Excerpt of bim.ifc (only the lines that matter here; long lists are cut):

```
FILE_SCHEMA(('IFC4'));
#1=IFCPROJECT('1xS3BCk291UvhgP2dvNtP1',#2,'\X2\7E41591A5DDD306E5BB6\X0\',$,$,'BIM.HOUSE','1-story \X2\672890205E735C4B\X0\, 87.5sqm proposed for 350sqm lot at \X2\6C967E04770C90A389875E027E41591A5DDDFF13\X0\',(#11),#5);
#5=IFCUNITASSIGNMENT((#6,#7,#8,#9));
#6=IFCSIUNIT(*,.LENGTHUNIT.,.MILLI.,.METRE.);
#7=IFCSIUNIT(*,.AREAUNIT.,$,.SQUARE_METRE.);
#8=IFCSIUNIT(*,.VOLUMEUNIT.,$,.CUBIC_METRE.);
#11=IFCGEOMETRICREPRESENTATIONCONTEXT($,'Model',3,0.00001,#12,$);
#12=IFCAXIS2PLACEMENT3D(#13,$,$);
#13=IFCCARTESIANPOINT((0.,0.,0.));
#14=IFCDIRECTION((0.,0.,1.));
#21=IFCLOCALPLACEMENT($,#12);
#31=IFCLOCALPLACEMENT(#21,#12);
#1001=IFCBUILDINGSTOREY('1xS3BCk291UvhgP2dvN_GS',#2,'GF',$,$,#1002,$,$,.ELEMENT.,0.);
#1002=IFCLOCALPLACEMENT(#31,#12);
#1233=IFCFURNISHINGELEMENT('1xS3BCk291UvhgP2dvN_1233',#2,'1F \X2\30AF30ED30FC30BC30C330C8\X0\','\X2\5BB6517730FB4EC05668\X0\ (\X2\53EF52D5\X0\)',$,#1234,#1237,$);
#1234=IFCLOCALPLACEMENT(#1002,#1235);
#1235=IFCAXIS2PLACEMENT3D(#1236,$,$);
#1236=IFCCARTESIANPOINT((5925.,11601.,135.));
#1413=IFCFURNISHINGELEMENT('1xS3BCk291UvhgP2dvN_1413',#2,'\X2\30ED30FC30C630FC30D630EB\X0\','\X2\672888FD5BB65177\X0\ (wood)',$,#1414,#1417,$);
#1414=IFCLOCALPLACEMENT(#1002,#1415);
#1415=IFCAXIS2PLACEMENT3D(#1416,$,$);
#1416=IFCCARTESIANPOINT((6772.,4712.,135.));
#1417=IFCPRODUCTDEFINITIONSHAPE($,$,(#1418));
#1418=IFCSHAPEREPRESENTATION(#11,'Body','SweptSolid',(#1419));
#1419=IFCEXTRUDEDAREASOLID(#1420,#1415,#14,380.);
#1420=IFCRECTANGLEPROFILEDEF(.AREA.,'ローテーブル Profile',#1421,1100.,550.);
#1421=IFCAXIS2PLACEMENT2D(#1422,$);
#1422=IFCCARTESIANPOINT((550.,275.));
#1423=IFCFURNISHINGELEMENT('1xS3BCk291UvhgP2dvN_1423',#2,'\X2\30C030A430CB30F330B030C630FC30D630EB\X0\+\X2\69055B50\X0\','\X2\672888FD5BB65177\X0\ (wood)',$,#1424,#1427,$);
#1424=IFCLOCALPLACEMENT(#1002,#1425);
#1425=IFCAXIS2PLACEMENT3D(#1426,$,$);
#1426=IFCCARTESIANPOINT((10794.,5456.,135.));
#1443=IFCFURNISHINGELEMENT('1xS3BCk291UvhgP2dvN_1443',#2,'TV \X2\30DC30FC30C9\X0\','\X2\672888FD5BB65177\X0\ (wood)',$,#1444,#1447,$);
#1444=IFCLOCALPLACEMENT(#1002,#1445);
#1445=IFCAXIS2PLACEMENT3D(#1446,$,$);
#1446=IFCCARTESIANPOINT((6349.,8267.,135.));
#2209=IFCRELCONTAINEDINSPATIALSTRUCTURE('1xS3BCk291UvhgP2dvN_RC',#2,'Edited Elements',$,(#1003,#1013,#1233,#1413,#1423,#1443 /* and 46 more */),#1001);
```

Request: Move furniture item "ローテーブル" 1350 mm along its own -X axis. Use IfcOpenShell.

```python
import ifcopenshell
import ifcopenshell.api.geometry
import ifcopenshell.util.placement

model = ifcopenshell.open("bim.ifc")

item = model.by_guid("1xS3BCk291UvhgP2dvN_1413")
matrix = ifcopenshell.util.placement.get_local_placement(item.ObjectPlacement)
matrix[:3, 3] -= matrix[:3, 0] * 1350.0
ifcopenshell.api.geometry.edit_object_placement(model, product=item, matrix=matrix, is_si=False)

print(ifcopenshell.util.placement.get_local_placement(item.ObjectPlacement).round(3) + 0.0)

model.write("bim_updated.ifc")
```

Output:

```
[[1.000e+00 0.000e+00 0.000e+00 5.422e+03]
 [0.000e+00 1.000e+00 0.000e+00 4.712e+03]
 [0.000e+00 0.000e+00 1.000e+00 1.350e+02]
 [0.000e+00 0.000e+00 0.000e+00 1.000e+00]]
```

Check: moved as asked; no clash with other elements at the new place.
